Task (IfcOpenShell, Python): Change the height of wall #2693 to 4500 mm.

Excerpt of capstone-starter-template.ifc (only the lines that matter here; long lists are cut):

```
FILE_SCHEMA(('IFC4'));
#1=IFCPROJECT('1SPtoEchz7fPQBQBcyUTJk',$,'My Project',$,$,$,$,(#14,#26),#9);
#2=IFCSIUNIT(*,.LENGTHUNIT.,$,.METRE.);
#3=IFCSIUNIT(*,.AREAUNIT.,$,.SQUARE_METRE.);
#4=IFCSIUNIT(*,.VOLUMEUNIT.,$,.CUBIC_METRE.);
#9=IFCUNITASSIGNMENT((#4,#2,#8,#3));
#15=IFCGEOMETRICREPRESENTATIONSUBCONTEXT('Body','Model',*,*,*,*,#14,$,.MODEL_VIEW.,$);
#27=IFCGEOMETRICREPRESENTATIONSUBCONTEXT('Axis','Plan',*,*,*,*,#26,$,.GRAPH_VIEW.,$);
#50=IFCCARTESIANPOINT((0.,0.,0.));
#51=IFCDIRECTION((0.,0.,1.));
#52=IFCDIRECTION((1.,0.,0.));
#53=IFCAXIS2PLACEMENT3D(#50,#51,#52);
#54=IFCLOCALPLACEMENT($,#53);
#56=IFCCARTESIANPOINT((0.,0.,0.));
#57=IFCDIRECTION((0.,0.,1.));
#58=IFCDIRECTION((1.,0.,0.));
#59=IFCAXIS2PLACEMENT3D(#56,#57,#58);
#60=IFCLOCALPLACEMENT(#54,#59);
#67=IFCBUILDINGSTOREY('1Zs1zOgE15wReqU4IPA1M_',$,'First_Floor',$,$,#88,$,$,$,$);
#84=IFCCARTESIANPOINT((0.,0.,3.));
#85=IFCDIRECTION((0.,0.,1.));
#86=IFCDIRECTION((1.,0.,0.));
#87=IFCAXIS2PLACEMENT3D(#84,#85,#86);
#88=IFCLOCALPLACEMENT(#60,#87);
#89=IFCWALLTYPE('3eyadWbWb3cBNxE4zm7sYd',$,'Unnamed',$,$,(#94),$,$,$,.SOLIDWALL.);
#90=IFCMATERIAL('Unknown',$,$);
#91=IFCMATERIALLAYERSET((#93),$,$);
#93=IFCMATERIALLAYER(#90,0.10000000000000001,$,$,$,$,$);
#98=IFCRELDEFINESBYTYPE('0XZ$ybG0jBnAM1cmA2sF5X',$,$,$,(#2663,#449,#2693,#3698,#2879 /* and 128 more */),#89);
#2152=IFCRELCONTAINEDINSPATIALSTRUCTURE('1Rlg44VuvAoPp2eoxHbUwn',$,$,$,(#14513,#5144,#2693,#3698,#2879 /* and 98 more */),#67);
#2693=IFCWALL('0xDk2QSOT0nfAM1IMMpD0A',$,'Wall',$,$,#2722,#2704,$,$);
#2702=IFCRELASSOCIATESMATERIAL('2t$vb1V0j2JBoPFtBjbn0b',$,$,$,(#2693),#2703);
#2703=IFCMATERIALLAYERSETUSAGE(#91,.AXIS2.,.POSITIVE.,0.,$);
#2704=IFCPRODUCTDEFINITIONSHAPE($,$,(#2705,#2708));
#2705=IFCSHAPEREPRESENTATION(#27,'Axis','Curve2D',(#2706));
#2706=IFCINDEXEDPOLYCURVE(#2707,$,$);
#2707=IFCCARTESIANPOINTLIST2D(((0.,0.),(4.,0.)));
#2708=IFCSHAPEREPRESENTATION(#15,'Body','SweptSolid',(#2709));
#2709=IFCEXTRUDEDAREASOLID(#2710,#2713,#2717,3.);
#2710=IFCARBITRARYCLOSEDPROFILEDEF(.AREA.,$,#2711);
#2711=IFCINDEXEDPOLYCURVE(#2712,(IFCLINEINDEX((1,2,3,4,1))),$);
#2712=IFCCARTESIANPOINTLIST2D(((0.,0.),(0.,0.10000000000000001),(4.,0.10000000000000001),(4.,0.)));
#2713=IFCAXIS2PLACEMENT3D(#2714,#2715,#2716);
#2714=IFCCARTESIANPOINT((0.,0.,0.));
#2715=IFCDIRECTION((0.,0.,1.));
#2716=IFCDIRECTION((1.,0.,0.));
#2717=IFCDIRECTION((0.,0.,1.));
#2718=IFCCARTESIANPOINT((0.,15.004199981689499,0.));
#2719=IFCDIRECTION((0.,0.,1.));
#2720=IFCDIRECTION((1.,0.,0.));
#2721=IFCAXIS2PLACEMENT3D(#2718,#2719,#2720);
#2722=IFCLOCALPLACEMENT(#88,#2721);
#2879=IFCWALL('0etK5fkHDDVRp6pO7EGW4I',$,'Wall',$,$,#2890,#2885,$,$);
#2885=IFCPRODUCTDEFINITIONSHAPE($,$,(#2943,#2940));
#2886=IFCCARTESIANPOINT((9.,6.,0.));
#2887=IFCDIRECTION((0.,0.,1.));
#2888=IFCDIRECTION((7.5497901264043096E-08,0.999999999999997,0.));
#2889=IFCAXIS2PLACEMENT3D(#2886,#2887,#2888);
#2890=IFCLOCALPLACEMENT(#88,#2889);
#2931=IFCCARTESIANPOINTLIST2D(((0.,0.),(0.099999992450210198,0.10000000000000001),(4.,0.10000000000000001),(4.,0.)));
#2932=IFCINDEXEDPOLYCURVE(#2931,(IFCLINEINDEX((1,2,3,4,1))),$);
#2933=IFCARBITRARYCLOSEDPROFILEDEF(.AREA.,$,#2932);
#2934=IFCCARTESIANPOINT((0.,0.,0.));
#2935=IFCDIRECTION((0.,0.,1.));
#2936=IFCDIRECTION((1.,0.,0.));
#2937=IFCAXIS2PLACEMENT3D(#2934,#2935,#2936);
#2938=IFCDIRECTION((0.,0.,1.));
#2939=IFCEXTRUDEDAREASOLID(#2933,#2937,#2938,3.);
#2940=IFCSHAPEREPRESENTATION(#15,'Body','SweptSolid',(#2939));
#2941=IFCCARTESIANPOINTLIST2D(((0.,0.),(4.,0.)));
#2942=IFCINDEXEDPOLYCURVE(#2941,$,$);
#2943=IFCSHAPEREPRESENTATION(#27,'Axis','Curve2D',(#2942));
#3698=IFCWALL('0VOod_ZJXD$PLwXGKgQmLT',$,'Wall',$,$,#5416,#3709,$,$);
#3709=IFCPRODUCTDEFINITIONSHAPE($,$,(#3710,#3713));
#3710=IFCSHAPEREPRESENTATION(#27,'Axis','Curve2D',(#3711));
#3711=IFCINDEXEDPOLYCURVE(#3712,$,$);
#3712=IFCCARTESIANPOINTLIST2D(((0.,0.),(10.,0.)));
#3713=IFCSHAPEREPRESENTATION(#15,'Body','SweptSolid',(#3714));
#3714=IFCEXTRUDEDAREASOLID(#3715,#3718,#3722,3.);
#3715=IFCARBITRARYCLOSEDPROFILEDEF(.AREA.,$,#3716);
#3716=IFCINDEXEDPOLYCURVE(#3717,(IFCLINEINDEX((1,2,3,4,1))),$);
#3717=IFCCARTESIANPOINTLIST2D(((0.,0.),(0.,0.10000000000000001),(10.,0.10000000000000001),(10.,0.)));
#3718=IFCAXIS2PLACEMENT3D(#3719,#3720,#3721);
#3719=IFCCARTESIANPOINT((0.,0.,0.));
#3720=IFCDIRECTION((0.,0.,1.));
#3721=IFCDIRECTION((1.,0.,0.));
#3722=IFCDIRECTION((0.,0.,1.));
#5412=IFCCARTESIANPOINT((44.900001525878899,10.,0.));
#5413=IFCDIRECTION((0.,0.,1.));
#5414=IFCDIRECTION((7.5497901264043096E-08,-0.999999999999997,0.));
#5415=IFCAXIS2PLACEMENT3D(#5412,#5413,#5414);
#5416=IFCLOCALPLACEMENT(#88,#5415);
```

```python
import ifcopenshell
import ifcopenshell.geom
import ifcopenshell.util.representation
import ifcopenshell.util.shape
import ifcopenshell.util.unit

model = ifcopenshell.open("capstone-starter-template.ifc")
unit_scale = ifcopenshell.util.unit.calculate_unit_scale(model)
settings = ifcopenshell.geom.settings()


def volume(element):
    """Net volume in cubic metres, openings subtracted."""
    shape = ifcopenshell.geom.create_shape(settings, element)
    return ifcopenshell.util.shape.get_volume(shape.geometry)


wall = model.by_guid("0xDk2QSOT0nfAM1IMMpD0A")
before = volume(wall)

body = ifcopenshell.util.representation.get_representation(wall, "Model", "Body")
solid = body.Items[0]
old_height = solid.Depth
solid.Depth = 4.5 / unit_scale
after = volume(wall)

print(f"height {old_height:g} -> {solid.Depth:g}, volume {before:.3f} -> {after:.3f} m3")

model.write("capstone-starter-template_updated.ifc")
```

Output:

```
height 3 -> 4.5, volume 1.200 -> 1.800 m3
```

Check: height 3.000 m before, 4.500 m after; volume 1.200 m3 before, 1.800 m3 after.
